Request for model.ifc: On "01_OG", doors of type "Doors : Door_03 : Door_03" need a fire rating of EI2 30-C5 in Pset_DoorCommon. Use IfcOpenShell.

First a look at what the model holds.

```python
import ifcopenshell
import ifcopenshell.util.element

model = ifcopenshell.open("model.ifc")
print(model.schema)
storey = next(s for s in model.by_type("IfcBuildingStorey") if s.Name == "01_OG")
doors = [e for e in ifcopenshell.util.element.get_decomposition(storey) if e.is_a("IfcDoor")]
seen = {}
for e in doors:
    element_type = ifcopenshell.util.element.get_type(e)
    key = (element_type.Name if element_type != e and element_type else None, ifcopenshell.util.element.get_pset(e, "Pset_DoorCommon", "FireRating"))
    seen[key] = seen.get(key, 0) + 1
for (name, value), count in sorted(seen.items(), key=str):
    print(count, "x", name, "|", value)
```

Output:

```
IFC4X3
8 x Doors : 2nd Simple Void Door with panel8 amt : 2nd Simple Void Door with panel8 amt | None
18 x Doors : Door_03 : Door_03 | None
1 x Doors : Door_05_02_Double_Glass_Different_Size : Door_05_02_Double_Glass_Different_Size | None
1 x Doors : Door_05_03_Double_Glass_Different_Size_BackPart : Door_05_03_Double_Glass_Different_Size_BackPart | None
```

```python
import ifcopenshell
import ifcopenshell.api.pset
import ifcopenshell.util.element

model = ifcopenshell.open("model.ifc")

storey = next(s for s in model.by_type("IfcBuildingStorey") if s.Name == "01_OG")
doors = [e for e in ifcopenshell.util.element.get_decomposition(storey) if e.is_a("IfcDoor")]

count = 0
for e in doors:
    element_type = ifcopenshell.util.element.get_type(e)
    if element_type in (None, e) or element_type.Name != "Doors : Door_03 : Door_03":
        continue
    # add_pset returns the element's existing set when there is one.
    pset = ifcopenshell.api.pset.add_pset(model, product=e, name="Pset_DoorCommon")
    ifcopenshell.api.pset.edit_pset(model, pset=pset, properties={"FireRating": "EI2 30-C5"})
    count += 1

print(count, "doors updated")

model.write("model-out.ifc")
```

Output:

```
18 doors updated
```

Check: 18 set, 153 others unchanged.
